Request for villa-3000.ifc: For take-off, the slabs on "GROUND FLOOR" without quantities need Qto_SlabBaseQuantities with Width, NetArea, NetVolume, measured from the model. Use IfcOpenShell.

First a look at what the model holds.

```python
import ifcopenshell
import ifcopenshell.util.element
import ifcopenshell.util.unit

model = ifcopenshell.open("villa-3000.ifc")
print(model.schema)
for unit_type in ("LENGTHUNIT", "AREAUNIT", "VOLUMEUNIT"):
    print(unit_type, ifcopenshell.util.unit.calculate_unit_scale(model, unit_type))
storey = next(s for s in model.by_type("IfcBuildingStorey") if s.Name == "GROUND FLOOR")
slabs = [e for e in ifcopenshell.util.element.get_decomposition(storey) if e.is_a("IfcSlab")]
for e in sorted(slabs, key=lambda e: e.id()):
    print(e.id(), e.is_a(), e.Name, list(ifcopenshell.util.element.get_psets(e, qtos_only=True)), sep=" | ")
```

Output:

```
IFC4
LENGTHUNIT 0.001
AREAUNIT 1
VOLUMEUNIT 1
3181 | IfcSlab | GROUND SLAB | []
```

```python
import ifcopenshell
import ifcopenshell.api.pset
import ifcopenshell.geom
import ifcopenshell.util.element
import ifcopenshell.util.shape
import ifcopenshell.util.unit

model = ifcopenshell.open("villa-3000.ifc")
unit_scale = ifcopenshell.util.unit.calculate_unit_scale(model)
area_scale = ifcopenshell.util.unit.calculate_unit_scale(model, "AREAUNIT")
volume_scale = ifcopenshell.util.unit.calculate_unit_scale(model, "VOLUMEUNIT")
settings = ifcopenshell.geom.settings()

storey = next(s for s in model.by_type("IfcBuildingStorey") if s.Name == "GROUND FLOOR")
slabs = [e for e in ifcopenshell.util.element.get_decomposition(storey) if e.is_a("IfcSlab")]

for e in sorted(slabs, key=lambda e: e.id()):
    if ifcopenshell.util.element.get_psets(e, qtos_only=True, should_inherit=False):
        continue
    # Geometry comes back in metres, in the element's own axes.
    shape = ifcopenshell.geom.create_shape(settings, e)
    values = {
        "Width": ifcopenshell.util.shape.get_z(shape.geometry) / unit_scale,
        "NetArea": ifcopenshell.util.shape.get_footprint_area(shape.geometry) / area_scale,
        "NetVolume": ifcopenshell.util.shape.get_volume(shape.geometry) / volume_scale,
    }
    qto = ifcopenshell.api.pset.add_qto(model, product=e, name="Qto_SlabBaseQuantities")
    ifcopenshell.api.pset.edit_qto(model, qto=qto, properties=values)
    print(e.id(), {k: round(v, 3) for k, v in values.items()})

model.write("villa-3000_updated.ifc")
```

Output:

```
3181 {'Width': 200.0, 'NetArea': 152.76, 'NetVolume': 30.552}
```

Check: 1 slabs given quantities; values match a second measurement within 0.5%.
